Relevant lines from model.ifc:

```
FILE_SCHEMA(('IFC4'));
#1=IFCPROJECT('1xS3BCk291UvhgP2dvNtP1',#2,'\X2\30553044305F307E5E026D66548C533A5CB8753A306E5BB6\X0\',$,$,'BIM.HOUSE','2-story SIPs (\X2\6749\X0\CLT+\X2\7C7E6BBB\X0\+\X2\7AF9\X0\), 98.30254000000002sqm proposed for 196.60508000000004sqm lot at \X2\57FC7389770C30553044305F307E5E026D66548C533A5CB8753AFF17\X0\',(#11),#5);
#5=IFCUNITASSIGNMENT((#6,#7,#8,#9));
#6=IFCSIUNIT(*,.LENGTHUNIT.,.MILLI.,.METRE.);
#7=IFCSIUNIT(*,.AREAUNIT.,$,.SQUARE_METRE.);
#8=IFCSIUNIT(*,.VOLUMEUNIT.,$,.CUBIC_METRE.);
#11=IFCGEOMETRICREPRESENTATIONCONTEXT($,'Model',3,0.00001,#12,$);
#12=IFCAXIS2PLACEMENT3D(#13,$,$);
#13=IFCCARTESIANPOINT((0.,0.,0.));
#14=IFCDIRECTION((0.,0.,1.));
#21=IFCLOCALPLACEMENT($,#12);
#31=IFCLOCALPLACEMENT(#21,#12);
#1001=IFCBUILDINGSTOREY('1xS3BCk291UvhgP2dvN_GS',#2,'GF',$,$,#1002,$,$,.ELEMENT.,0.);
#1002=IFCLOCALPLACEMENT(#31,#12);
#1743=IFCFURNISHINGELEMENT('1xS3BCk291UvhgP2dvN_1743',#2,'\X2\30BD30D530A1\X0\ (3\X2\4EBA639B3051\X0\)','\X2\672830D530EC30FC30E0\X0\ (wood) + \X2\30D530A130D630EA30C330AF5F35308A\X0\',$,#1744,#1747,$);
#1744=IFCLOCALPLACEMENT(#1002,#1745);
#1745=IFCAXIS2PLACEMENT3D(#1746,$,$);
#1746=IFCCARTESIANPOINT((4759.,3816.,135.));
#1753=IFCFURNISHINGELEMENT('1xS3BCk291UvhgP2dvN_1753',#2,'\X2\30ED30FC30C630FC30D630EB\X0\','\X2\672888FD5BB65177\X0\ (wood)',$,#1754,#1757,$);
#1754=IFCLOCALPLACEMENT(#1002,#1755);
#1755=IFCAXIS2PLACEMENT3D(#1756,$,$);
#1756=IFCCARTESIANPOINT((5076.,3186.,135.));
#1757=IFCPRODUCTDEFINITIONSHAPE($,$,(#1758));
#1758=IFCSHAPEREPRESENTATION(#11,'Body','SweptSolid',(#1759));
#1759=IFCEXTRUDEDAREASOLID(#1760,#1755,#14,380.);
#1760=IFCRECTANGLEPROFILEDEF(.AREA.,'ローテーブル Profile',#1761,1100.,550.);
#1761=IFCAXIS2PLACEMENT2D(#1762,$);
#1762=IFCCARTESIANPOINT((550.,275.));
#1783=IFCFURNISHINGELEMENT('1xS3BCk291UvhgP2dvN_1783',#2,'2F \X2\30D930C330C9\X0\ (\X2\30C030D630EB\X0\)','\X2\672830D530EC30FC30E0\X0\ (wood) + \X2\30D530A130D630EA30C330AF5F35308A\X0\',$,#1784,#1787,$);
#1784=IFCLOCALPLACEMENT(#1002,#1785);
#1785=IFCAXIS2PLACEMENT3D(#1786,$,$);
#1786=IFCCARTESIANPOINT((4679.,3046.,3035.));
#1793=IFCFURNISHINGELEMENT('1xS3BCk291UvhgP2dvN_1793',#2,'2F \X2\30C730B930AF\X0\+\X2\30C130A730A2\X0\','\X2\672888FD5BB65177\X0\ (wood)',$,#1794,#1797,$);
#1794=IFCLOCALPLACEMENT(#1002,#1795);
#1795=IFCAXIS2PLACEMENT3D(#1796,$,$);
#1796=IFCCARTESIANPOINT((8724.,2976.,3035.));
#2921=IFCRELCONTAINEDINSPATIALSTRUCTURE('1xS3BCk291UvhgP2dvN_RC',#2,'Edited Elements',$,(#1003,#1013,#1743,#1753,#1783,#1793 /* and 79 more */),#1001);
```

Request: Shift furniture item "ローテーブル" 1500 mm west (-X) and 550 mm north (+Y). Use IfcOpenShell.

```python
import ifcopenshell
import ifcopenshell.api.geometry
import ifcopenshell.util.placement

model = ifcopenshell.open("model.ifc")

item = model.by_guid("1xS3BCk291UvhgP2dvN_1753")
matrix = ifcopenshell.util.placement.get_local_placement(item.ObjectPlacement)
matrix[0, 3] -= 1500.0
matrix[1, 3] += 550.0
ifcopenshell.api.geometry.edit_object_placement(model, product=item, matrix=matrix, is_si=False)

print(ifcopenshell.util.placement.get_local_placement(item.ObjectPlacement).round(3) + 0.0)

model.write("model_edited.ifc")
```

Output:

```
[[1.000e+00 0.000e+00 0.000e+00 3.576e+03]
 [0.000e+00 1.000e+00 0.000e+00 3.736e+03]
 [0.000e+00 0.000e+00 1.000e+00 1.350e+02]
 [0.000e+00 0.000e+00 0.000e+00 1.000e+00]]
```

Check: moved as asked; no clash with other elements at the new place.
